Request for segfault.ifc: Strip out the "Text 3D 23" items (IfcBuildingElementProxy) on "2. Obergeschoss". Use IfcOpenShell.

First a look at what the model holds.

```python
import ifcopenshell
import ifcopenshell.util.element

model = ifcopenshell.open("segfault.ifc")
print(model.schema)
storey = next(s for s in model.by_type("IfcBuildingStorey") if s.Name == "2. Obergeschoss")
proxies = [e for e in ifcopenshell.util.element.get_decomposition(storey) if e.is_a("IfcBuildingElementProxy")]
seen = {}
for e in proxies:
    element_type = ifcopenshell.util.element.get_type(e)
    name = element_type.Name if element_type not in (None, e) else None
    seen[name] = seen.get(name, 0) + 1
for name, count in sorted(seen.items(), key=str):
    print(count, "x", name)
```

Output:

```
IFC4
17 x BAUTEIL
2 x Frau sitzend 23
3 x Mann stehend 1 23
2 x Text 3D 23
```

```python
import ifcopenshell
import ifcopenshell.api.root
import ifcopenshell.util.element

model = ifcopenshell.open("segfault.ifc")

storey = next(s for s in model.by_type("IfcBuildingStorey") if s.Name == "2. Obergeschoss")
proxies = [e for e in ifcopenshell.util.element.get_decomposition(storey) if e.is_a("IfcBuildingElementProxy")]
targets = [e for e in proxies if (t := ifcopenshell.util.element.get_type(e)) not in (None, e) and t.Name == "Text 3D 23"]

for e in targets:
    ifcopenshell.api.root.remove_product(model, product=e)
print(len(targets), "removed")

model.write("segfault_v2.ifc")
```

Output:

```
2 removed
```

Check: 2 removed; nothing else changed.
